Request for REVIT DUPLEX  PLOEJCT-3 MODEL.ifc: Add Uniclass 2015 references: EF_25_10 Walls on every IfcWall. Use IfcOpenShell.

First a look at what the model holds.

```python
import ifcopenshell

model = ifcopenshell.open("REVIT DUPLEX  PLOEJCT-3 MODEL.ifc")
print(model.schema)
print("classifications:", [c.Name for c in model.by_type("IfcClassification")])
for ifc_class in ("IfcDoor", "IfcRoof", "IfcStair", "IfcWall", "IfcWindow"):
    print(ifc_class, len(model.by_type(ifc_class)))
```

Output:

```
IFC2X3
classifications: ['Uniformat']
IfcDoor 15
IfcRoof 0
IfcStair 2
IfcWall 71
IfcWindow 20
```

```python
import ifcopenshell
import ifcopenshell.api.classification

model = ifcopenshell.open("REVIT DUPLEX  PLOEJCT-3 MODEL.ifc")

# IFC2X3 requires Source and Edition and has no link from the project to the system.
system = model.create_entity("IfcClassification", Source="NBS", Edition="2015", Name="Uniclass 2015")

codes = {
    "IfcWall": ("EF_25_10", "Walls"),
}
for ifc_class, (code, name) in codes.items():
    products = model.by_type(ifc_class)
    ifcopenshell.api.classification.add_reference(
        model, products=products, classification=system, identification=code, name=name
    )
    print(code, len(products))

model.write("REVIT DUPLEX  PLOEJCT-3 MODEL_v2.ifc")
```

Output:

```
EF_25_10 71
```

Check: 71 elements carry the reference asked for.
